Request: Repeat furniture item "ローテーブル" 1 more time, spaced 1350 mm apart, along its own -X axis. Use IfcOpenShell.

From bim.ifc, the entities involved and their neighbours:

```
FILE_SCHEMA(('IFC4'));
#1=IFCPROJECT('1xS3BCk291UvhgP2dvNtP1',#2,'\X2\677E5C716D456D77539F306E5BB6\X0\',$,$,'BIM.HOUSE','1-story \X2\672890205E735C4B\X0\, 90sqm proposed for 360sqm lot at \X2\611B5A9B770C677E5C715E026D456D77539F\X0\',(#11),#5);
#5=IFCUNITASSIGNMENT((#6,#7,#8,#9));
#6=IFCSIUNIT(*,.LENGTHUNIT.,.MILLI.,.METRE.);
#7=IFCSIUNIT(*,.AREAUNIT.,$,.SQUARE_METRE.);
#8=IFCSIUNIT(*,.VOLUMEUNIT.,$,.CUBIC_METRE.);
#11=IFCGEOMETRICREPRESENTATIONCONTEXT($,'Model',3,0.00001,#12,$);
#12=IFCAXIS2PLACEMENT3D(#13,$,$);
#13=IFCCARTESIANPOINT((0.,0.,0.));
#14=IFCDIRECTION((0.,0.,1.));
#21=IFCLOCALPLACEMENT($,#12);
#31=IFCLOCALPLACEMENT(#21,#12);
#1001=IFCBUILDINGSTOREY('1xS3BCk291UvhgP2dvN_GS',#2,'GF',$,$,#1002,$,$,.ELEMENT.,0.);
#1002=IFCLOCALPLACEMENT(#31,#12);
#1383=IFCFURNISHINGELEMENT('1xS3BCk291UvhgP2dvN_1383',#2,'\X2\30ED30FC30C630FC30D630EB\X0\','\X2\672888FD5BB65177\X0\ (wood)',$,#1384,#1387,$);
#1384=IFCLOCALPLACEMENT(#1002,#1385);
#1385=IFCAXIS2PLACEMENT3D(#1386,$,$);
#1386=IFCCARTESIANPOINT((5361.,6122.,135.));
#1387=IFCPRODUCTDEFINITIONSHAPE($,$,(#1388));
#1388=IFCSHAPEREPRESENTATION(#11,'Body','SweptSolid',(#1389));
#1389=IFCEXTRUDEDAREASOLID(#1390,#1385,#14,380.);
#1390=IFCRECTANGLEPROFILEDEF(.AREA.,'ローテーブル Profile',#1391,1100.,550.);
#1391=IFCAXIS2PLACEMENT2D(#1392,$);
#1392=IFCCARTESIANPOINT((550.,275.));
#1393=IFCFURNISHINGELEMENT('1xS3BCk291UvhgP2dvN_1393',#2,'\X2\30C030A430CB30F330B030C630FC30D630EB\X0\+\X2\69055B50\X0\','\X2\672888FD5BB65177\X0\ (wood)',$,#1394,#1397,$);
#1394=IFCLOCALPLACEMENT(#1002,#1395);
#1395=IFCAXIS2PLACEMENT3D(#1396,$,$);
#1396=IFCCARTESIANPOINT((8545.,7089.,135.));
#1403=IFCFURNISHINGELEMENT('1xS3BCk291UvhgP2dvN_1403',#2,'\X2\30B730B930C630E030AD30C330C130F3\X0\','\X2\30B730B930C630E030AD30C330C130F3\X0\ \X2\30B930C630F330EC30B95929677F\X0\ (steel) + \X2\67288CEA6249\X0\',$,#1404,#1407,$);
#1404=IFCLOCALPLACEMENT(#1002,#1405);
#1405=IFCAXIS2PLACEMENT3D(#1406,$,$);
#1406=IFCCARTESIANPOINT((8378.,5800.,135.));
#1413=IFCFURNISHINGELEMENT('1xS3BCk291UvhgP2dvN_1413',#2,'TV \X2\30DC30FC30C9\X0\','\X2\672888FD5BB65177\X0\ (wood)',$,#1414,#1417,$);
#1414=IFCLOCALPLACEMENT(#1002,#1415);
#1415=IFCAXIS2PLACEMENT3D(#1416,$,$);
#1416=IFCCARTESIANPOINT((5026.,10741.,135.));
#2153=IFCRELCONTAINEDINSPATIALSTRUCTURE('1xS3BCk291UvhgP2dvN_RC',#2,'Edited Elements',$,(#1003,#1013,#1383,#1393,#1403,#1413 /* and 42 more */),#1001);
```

```python
import ifcopenshell
import ifcopenshell.api.geometry
import ifcopenshell.api.root
import ifcopenshell.util.element
import ifcopenshell.util.placement

model = ifcopenshell.open("bim.ifc")


def reuse_history(source, copy):
    """copy_class also copies each property set's owner history, people and application; keep the originals."""
    for rel in copy.IsDefinedBy:
        if rel.is_a("IfcRelDefinesByProperties") and (history := rel.RelatingPropertyDefinition.OwnerHistory):
            rel.RelatingPropertyDefinition.OwnerHistory = source.OwnerHistory
            ifcopenshell.util.element.remove_deep2(model, history)


source = model.by_guid("1xS3BCk291UvhgP2dvN_1383")
base = ifcopenshell.util.placement.get_local_placement(source.ObjectPlacement)
step = -base[:3, 0] * 1350.0

for i in range(1, 2):
    copy = ifcopenshell.api.root.copy_class(model, product=source)
    copy.Representation = ifcopenshell.util.element.copy_deep(
        model, source.Representation, exclude=["IfcGeometricRepresentationContext", "IfcRepresentationMap"]
    )
    reuse_history(source, copy)
    matrix = base.copy()
    matrix[:3, 3] += i * step
    print("added at", matrix[:3, 3].round(3) + 0.0)
    ifcopenshell.api.geometry.edit_object_placement(model, product=copy, matrix=matrix, is_si=False)

model.write("bim_updated.ifc")
```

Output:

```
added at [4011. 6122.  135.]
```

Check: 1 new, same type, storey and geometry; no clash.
